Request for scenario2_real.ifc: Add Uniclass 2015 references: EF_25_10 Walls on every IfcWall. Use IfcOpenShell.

First a look at what the model holds.

```python
import ifcopenshell

model = ifcopenshell.open("scenario2_real.ifc")
print(model.schema)
print("classifications:", [c.Name for c in model.by_type("IfcClassification")])
for ifc_class in ("IfcDoor", "IfcRoof", "IfcStair", "IfcWall", "IfcWindow"):
    print(ifc_class, len(model.by_type(ifc_class)))
```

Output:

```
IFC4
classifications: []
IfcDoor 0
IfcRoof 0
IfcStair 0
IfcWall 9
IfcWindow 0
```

```python
import ifcopenshell
import ifcopenshell.api.classification

model = ifcopenshell.open("scenario2_real.ifc")

system = ifcopenshell.api.classification.add_classification(model, classification="Uniclass 2015")

codes = {
    "IfcWall": ("EF_25_10", "Walls"),
}
for ifc_class, (code, name) in codes.items():
    products = model.by_type(ifc_class)
    ifcopenshell.api.classification.add_reference(
        model, products=products, classification=system, identification=code, name=name
    )
    print(code, len(products))

model.write("scenario2_real_rev.ifc")
```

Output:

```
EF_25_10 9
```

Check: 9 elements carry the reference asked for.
